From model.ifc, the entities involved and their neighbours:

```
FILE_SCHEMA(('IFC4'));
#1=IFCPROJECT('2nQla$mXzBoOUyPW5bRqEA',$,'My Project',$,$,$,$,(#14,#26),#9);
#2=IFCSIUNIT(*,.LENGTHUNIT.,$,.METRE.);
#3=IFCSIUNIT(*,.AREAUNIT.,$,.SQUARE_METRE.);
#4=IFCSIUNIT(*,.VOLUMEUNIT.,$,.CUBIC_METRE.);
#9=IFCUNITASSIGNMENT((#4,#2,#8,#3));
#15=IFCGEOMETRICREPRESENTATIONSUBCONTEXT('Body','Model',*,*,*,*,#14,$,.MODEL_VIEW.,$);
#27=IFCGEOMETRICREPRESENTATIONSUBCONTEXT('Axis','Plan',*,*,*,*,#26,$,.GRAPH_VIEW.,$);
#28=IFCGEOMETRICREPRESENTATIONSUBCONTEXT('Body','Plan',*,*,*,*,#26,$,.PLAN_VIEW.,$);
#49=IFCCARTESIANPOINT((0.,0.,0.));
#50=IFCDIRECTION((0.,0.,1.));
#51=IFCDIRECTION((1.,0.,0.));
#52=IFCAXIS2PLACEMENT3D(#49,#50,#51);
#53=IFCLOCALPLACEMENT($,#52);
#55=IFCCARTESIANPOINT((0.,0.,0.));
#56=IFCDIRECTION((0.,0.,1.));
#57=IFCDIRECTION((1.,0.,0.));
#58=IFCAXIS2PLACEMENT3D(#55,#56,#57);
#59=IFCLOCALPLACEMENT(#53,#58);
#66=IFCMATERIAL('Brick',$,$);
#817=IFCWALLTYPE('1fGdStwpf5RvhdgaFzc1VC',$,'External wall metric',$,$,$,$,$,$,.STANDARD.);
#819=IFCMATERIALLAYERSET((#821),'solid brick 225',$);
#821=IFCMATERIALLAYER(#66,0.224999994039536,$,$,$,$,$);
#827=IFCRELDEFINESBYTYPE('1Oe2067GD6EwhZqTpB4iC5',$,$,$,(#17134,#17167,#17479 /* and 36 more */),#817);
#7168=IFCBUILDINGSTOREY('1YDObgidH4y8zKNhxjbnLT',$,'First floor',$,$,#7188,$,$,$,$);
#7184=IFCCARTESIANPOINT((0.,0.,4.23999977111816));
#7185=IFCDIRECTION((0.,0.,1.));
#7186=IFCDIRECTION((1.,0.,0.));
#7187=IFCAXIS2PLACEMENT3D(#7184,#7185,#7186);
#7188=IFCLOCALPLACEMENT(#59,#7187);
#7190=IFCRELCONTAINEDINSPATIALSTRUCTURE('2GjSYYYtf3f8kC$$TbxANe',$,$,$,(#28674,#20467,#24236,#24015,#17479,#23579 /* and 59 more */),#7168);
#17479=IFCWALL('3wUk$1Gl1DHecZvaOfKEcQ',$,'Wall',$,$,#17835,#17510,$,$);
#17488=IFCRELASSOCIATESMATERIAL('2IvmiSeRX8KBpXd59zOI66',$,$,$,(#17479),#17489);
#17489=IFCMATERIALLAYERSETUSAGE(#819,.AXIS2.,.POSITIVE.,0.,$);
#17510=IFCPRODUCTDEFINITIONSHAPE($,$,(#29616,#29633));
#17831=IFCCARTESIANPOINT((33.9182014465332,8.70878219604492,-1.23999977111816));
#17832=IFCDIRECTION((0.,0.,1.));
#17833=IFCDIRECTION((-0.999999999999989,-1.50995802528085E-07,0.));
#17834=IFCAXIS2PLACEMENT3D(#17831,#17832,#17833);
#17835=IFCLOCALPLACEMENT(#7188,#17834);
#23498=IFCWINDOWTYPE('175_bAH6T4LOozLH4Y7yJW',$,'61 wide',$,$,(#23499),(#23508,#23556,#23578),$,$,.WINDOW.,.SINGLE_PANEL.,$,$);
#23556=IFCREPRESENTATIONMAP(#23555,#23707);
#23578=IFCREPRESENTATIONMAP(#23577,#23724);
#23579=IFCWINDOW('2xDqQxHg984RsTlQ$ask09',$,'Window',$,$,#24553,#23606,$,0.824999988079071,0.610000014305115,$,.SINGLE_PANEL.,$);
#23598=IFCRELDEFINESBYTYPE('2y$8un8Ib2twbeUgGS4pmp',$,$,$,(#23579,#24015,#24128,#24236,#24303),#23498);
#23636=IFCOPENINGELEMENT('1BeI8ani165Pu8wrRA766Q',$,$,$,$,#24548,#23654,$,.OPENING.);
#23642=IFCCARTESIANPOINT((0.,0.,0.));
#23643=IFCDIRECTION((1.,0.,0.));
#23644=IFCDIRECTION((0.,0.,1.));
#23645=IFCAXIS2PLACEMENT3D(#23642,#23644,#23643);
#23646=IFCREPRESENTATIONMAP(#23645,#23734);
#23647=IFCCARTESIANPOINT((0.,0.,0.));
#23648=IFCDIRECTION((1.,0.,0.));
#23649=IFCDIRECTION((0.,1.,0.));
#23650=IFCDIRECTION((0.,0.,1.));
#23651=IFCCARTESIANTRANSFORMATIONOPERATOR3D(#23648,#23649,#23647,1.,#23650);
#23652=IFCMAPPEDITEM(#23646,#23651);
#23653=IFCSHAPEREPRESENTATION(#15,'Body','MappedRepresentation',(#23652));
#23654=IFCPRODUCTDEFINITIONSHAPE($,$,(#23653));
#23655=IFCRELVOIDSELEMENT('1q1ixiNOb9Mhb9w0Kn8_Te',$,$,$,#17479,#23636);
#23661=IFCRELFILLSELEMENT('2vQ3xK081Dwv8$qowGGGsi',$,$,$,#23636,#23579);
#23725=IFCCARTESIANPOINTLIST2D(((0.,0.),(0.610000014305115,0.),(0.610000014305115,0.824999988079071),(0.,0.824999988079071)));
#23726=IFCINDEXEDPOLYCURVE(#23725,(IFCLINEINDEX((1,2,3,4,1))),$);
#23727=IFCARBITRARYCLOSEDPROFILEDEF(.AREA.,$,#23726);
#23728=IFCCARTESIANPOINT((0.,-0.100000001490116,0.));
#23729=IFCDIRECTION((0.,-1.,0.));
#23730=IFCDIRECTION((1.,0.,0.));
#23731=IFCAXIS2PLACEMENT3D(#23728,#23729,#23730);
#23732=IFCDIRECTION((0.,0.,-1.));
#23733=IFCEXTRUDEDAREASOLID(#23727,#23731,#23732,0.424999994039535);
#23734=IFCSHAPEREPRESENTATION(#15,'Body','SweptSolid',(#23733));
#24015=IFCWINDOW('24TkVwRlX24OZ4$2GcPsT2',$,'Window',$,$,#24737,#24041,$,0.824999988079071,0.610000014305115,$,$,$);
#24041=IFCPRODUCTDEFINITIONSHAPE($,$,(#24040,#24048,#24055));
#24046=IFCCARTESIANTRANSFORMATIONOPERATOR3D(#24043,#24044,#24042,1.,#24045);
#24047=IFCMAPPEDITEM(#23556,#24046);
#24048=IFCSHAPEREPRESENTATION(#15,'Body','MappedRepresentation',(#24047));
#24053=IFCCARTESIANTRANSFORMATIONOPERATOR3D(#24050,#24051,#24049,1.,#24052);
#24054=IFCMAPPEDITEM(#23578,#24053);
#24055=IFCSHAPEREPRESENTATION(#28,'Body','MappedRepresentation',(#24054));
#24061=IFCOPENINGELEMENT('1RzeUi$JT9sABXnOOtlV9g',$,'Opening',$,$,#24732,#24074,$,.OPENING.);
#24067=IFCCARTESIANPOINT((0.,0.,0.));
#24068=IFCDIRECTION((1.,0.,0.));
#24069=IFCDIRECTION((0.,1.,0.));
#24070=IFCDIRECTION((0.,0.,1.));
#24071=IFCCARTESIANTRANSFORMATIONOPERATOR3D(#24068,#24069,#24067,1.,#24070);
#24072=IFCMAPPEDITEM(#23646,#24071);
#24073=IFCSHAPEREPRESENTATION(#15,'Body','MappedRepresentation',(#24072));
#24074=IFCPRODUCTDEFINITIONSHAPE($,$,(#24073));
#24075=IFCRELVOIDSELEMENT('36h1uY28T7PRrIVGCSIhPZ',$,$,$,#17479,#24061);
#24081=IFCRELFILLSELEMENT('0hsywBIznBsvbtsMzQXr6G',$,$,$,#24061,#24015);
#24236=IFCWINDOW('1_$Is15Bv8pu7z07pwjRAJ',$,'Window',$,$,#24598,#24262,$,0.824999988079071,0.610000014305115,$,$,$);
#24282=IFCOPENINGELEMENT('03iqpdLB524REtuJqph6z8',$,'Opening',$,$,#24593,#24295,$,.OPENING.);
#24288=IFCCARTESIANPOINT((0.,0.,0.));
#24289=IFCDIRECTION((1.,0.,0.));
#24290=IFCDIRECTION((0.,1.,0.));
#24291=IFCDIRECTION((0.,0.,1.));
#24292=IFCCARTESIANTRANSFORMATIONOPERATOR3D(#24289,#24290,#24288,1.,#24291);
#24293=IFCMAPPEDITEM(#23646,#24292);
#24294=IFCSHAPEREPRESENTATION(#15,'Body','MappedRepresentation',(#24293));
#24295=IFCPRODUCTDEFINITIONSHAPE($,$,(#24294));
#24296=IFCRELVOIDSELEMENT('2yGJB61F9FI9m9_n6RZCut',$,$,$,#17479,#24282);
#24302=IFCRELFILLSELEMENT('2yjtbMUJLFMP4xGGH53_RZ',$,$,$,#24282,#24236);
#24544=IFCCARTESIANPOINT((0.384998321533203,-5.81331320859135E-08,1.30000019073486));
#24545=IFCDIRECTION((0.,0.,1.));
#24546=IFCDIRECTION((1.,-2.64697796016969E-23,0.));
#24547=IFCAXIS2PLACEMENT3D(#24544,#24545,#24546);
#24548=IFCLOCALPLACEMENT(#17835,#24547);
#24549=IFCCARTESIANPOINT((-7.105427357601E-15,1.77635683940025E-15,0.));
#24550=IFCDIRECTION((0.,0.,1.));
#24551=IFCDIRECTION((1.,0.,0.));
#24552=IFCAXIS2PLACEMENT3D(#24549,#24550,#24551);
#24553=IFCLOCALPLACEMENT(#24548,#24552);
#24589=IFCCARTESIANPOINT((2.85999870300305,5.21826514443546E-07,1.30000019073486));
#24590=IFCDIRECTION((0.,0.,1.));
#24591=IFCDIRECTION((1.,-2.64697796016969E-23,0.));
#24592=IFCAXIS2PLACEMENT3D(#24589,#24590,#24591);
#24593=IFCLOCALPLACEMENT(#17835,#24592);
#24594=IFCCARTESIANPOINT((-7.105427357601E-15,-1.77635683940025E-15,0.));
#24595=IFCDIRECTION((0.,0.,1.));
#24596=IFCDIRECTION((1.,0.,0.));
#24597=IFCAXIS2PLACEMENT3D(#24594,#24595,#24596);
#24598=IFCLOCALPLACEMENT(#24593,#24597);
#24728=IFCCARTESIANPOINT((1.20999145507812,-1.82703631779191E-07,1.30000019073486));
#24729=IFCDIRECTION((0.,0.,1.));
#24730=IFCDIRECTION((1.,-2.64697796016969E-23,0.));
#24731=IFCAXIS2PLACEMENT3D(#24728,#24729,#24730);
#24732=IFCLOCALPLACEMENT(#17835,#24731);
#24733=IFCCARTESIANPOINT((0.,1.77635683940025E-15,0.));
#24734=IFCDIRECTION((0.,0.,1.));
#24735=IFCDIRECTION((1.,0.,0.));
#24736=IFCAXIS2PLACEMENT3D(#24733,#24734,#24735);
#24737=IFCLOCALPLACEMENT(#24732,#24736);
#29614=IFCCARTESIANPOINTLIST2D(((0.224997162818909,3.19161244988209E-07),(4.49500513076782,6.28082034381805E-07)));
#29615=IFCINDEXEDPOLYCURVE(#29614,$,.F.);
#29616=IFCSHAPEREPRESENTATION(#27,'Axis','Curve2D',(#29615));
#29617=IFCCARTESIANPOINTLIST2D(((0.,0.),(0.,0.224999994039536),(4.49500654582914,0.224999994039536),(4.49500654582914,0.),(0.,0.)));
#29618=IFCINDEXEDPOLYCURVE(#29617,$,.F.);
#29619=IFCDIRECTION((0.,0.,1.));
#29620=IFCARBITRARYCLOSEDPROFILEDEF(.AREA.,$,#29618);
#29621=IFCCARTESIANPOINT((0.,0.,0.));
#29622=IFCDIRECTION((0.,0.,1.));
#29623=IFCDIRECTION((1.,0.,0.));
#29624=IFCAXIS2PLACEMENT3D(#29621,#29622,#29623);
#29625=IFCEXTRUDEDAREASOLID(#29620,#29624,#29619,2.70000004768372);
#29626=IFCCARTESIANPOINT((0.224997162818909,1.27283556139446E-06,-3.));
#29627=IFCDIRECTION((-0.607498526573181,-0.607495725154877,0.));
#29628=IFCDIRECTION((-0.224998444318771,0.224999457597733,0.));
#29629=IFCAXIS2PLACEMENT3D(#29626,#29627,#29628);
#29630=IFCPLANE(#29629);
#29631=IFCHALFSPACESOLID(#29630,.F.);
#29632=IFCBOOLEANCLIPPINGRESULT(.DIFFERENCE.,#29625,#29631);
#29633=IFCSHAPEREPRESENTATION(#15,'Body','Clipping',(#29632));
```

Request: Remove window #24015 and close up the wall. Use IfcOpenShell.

```python
import ifcopenshell
import ifcopenshell.api.feature
import ifcopenshell.api.root
import ifcopenshell.geom
import ifcopenshell.util.shape

model = ifcopenshell.open("model.ifc")
settings = ifcopenshell.geom.settings()


def volume(element):
    """Net volume in cubic metres, openings subtracted."""
    shape = ifcopenshell.geom.create_shape(settings, element)
    return ifcopenshell.util.shape.get_volume(shape.geometry)


window = model.by_guid("24TkVwRlX24OZ4$2GcPsT2")
opening = window.FillsVoids[0].RelatingOpeningElement
wall = opening.VoidsElements[0].RelatingBuildingElement
before = volume(wall)

ifcopenshell.api.root.remove_product(model, product=window)
ifcopenshell.api.feature.remove_feature(model, feature=opening)

after = volume(wall)

print(f"wall volume {before:.3f} -> {after:.3f} m3")

model.write("model_updated.ifc")
```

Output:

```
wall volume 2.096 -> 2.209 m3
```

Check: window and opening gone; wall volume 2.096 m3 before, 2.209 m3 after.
